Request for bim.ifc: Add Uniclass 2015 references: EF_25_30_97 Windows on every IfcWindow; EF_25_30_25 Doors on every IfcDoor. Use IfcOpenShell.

First a look at what the model holds.

```python
import ifcopenshell

model = ifcopenshell.open("bim.ifc")
print(model.schema)
print("classifications:", [c.Name for c in model.by_type("IfcClassification")])
for ifc_class in ("IfcDoor", "IfcRoof", "IfcStair", "IfcWall", "IfcWindow"):
    print(ifc_class, len(model.by_type(ifc_class)))
```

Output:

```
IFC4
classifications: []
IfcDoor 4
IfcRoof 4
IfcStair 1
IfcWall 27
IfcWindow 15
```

```python
import ifcopenshell
import ifcopenshell.api.classification

model = ifcopenshell.open("bim.ifc")

system = ifcopenshell.api.classification.add_classification(model, classification="Uniclass 2015")

codes = {
    "IfcWindow": ("EF_25_30_97", "Windows"),
    "IfcDoor": ("EF_25_30_25", "Doors"),
}
for ifc_class, (code, name) in codes.items():
    products = model.by_type(ifc_class)
    ifcopenshell.api.classification.add_reference(
        model, products=products, classification=system, identification=code, name=name
    )
    print(code, len(products))

model.write("bim-out.ifc")
```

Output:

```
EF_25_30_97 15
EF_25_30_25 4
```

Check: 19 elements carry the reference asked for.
